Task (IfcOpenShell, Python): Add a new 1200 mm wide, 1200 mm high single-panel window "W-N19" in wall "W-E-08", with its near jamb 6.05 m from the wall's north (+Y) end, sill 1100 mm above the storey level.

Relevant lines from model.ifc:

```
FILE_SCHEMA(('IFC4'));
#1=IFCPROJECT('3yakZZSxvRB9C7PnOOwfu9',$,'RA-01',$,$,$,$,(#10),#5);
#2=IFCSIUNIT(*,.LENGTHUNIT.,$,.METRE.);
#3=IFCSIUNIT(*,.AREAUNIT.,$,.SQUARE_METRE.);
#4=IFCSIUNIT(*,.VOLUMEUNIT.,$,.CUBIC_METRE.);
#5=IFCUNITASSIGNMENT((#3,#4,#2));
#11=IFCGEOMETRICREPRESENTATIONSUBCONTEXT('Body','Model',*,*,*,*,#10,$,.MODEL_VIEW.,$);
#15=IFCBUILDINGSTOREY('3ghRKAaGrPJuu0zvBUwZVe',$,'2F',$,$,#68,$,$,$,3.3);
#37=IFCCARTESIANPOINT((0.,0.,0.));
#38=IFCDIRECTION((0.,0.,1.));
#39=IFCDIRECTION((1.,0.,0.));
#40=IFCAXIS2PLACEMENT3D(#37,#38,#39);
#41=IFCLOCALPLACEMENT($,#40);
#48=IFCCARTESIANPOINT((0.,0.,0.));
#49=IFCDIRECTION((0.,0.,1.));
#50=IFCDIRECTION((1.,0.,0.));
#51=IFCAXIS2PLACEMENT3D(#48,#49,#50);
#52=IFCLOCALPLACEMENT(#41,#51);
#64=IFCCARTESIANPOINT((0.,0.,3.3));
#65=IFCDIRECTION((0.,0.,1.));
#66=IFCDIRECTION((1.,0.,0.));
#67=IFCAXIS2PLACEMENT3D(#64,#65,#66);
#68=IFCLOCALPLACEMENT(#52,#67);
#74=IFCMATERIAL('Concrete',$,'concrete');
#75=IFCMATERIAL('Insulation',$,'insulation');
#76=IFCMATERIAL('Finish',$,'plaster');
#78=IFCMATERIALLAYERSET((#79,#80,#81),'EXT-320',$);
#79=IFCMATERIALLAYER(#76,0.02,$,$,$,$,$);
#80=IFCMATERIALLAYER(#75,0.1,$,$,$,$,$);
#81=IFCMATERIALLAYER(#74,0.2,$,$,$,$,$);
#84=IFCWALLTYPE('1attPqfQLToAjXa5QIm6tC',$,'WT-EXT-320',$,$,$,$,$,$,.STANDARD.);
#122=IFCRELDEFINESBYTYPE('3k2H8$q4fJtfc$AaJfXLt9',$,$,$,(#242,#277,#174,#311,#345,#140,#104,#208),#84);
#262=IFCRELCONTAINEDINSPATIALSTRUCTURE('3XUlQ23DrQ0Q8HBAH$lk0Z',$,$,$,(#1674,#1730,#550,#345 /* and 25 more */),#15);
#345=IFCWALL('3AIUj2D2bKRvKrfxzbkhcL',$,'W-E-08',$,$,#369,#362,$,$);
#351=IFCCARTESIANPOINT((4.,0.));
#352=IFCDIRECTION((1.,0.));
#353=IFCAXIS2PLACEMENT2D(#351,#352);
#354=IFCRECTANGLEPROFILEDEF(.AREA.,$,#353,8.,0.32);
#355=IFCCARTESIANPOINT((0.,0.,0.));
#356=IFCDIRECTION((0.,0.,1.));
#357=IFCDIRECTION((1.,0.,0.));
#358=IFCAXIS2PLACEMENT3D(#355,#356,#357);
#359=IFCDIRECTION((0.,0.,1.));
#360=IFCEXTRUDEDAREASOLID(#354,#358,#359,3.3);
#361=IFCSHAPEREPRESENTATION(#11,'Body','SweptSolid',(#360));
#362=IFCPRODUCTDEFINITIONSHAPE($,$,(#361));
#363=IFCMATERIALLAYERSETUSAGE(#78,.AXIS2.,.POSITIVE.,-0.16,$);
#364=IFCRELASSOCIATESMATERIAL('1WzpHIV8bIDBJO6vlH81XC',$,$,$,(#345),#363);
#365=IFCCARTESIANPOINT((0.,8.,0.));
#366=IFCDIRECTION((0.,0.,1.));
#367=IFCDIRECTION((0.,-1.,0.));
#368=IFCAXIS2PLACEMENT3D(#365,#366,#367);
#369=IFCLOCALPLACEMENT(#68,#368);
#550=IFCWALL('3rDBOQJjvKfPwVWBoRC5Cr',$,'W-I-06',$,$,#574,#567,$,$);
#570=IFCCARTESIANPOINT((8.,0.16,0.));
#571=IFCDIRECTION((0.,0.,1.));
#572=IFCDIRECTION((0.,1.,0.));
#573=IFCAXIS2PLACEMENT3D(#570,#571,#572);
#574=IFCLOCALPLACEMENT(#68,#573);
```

```python
import numpy as np
import ifcopenshell
import ifcopenshell.api.feature
import ifcopenshell.api.geometry
import ifcopenshell.api.root
import ifcopenshell.api.spatial
import ifcopenshell.geom
import ifcopenshell.util.element
import ifcopenshell.util.placement
import ifcopenshell.util.representation
import ifcopenshell.util.shape
import ifcopenshell.util.unit

model = ifcopenshell.open("model.ifc")
unit_scale = ifcopenshell.util.unit.calculate_unit_scale(model)
settings = ifcopenshell.geom.settings()


def volume(element):
    """Net volume in cubic metres, openings subtracted."""
    shape = ifcopenshell.geom.create_shape(settings, element)
    return ifcopenshell.util.shape.get_volume(shape.geometry)


wall = model.by_guid("3AIUj2D2bKRvKrfxzbkhcL")
storey = ifcopenshell.util.element.get_container(wall, ifc_class="IfcBuildingStorey")
context = ifcopenshell.util.representation.get_context(model, "Model", "Body", "MODEL_VIEW")
before = volume(wall)

width, height, from_end, sill = 1.2, 1.2, 6.05, 1.1  # metres

# The wall runs along its own X axis, and the end named is its -X end.
wall_shape = ifcopenshell.geom.create_shape(settings, wall)
x, y, z = ifcopenshell.util.shape.get_vertices(wall_shape.geometry).T
start = x.min() + from_end
face, thickness = float(y.min()), float(y.max() - y.min())
wall_matrix = ifcopenshell.util.placement.get_local_placement(wall.ObjectPlacement)
level = ifcopenshell.util.placement.get_local_placement(storey.ObjectPlacement)[2, 3]


def in_wall(x, y):
    """Placement at x, y metres in the wall's axes, at sill height."""
    matrix = wall_matrix.copy()
    matrix[:, 3] = wall_matrix @ np.array([x / unit_scale, y / unit_scale, 0.0, 1.0])
    matrix[2, 3] = level + sill / unit_scale
    return matrix


# Opening: a box that overshoots both wall faces by 50 mm.
opening = ifcopenshell.api.root.create_entity(model, ifc_class="IfcOpeningElement", predefined_type="OPENING")
box = ifcopenshell.api.geometry.add_wall_representation(
    model, context=context, length=width, height=height, thickness=thickness + 0.1
)
ifcopenshell.api.geometry.assign_representation(model, product=opening, representation=box)
ifcopenshell.api.geometry.edit_object_placement(model, product=opening, matrix=in_wall(start, face - 0.05), is_si=False)
ifcopenshell.api.feature.add_feature(model, feature=opening, element=wall)

window = ifcopenshell.api.root.create_entity(model, ifc_class="IfcWindow", name="W-N19", predefined_type="WINDOW")
window.OverallWidth, window.OverallHeight = width / unit_scale, height / unit_scale
window.PartitioningType = "SINGLE_PANEL"
body = ifcopenshell.api.geometry.add_window_representation(
    model,
    context=context,
    overall_width=window.OverallWidth,
    overall_height=window.OverallHeight,
    partition_type="SINGLE_PANEL",
)
ifcopenshell.api.geometry.assign_representation(model, product=window, representation=body)
ifcopenshell.api.spatial.assign_container(model, products=[window], relating_structure=storey)
ifcopenshell.api.feature.add_filling(model, opening=opening, element=window)

# Centre the window in the wall's thickness.
ifcopenshell.api.geometry.edit_object_placement(model, product=window, matrix=in_wall(start, face), is_si=False)
window_shape = ifcopenshell.geom.create_shape(settings, window)
depth = ifcopenshell.util.shape.get_vertices(window_shape.geometry)[:, 1]
offset = face + thickness / 2 - (depth.min() + depth.max()) / 2
ifcopenshell.api.geometry.edit_object_placement(model, product=window, matrix=in_wall(start, offset), is_si=False)

after = volume(wall)

print(f"wall volume {before:.3f} -> {after:.3f} m3")

model.write("model-out.ifc")
```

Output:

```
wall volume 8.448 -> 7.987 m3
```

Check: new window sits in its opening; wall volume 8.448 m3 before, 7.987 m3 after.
